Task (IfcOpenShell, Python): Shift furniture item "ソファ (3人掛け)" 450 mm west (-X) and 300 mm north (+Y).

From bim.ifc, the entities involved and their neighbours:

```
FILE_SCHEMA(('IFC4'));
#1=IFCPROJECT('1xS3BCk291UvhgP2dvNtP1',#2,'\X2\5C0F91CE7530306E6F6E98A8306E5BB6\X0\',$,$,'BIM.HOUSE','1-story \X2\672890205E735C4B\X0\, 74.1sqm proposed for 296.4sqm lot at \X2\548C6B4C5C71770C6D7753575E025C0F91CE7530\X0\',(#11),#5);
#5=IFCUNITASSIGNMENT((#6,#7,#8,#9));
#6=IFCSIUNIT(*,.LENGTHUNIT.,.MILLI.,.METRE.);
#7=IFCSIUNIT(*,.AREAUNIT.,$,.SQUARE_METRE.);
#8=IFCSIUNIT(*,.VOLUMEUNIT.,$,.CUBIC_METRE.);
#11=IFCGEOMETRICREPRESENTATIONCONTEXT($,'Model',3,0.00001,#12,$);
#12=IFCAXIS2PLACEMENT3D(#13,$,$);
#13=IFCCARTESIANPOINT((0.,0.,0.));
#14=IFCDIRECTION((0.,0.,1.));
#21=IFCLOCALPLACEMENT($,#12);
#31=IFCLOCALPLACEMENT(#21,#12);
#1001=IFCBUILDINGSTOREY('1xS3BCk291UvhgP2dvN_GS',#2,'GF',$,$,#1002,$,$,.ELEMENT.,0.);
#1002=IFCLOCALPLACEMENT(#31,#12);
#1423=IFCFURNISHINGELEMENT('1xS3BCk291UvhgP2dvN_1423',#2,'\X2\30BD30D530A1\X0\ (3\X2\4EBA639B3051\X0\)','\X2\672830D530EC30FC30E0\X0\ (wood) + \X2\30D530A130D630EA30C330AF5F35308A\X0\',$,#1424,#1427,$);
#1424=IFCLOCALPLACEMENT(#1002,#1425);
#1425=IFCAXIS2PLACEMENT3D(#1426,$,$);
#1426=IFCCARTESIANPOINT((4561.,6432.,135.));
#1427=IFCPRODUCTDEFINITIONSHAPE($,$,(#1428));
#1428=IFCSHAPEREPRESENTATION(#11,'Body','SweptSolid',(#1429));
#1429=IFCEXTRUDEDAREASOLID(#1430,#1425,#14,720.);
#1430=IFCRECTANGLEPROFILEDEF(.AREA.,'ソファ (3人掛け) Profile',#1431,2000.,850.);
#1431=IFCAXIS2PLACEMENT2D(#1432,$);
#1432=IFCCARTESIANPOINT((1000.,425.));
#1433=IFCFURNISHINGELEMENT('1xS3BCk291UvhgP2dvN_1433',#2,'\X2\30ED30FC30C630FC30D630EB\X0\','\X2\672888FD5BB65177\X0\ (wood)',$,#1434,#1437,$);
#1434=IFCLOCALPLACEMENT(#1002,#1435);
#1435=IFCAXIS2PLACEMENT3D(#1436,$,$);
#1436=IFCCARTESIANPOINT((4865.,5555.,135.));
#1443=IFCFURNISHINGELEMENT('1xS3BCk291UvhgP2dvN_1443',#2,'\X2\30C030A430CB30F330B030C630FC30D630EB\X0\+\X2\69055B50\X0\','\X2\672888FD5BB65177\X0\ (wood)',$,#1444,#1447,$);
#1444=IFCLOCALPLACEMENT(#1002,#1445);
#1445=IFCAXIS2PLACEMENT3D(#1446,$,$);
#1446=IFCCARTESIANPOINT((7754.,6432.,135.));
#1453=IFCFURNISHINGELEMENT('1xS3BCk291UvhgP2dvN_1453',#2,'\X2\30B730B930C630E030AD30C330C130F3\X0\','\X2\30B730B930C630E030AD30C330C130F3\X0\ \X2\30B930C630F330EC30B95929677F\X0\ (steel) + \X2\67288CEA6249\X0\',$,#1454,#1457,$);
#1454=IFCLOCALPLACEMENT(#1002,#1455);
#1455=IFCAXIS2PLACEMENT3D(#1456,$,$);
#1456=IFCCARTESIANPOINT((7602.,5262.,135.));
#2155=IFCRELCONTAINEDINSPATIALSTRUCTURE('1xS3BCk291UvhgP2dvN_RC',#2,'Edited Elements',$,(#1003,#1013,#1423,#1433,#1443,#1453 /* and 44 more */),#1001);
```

```python
import ifcopenshell
import ifcopenshell.api.geometry
import ifcopenshell.util.placement

model = ifcopenshell.open("bim.ifc")

item = model.by_id(1423)
matrix = ifcopenshell.util.placement.get_local_placement(item.ObjectPlacement)
matrix[0, 3] -= 450.0
matrix[1, 3] += 300.0
ifcopenshell.api.geometry.edit_object_placement(model, product=item, matrix=matrix, is_si=False)

print(ifcopenshell.util.placement.get_local_placement(item.ObjectPlacement).round(3) + 0.0)

model.write("bim_rev.ifc")
```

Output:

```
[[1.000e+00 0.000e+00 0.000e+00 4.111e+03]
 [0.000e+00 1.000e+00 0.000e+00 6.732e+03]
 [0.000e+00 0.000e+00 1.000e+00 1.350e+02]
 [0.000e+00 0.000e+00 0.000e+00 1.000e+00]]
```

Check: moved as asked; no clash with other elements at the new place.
